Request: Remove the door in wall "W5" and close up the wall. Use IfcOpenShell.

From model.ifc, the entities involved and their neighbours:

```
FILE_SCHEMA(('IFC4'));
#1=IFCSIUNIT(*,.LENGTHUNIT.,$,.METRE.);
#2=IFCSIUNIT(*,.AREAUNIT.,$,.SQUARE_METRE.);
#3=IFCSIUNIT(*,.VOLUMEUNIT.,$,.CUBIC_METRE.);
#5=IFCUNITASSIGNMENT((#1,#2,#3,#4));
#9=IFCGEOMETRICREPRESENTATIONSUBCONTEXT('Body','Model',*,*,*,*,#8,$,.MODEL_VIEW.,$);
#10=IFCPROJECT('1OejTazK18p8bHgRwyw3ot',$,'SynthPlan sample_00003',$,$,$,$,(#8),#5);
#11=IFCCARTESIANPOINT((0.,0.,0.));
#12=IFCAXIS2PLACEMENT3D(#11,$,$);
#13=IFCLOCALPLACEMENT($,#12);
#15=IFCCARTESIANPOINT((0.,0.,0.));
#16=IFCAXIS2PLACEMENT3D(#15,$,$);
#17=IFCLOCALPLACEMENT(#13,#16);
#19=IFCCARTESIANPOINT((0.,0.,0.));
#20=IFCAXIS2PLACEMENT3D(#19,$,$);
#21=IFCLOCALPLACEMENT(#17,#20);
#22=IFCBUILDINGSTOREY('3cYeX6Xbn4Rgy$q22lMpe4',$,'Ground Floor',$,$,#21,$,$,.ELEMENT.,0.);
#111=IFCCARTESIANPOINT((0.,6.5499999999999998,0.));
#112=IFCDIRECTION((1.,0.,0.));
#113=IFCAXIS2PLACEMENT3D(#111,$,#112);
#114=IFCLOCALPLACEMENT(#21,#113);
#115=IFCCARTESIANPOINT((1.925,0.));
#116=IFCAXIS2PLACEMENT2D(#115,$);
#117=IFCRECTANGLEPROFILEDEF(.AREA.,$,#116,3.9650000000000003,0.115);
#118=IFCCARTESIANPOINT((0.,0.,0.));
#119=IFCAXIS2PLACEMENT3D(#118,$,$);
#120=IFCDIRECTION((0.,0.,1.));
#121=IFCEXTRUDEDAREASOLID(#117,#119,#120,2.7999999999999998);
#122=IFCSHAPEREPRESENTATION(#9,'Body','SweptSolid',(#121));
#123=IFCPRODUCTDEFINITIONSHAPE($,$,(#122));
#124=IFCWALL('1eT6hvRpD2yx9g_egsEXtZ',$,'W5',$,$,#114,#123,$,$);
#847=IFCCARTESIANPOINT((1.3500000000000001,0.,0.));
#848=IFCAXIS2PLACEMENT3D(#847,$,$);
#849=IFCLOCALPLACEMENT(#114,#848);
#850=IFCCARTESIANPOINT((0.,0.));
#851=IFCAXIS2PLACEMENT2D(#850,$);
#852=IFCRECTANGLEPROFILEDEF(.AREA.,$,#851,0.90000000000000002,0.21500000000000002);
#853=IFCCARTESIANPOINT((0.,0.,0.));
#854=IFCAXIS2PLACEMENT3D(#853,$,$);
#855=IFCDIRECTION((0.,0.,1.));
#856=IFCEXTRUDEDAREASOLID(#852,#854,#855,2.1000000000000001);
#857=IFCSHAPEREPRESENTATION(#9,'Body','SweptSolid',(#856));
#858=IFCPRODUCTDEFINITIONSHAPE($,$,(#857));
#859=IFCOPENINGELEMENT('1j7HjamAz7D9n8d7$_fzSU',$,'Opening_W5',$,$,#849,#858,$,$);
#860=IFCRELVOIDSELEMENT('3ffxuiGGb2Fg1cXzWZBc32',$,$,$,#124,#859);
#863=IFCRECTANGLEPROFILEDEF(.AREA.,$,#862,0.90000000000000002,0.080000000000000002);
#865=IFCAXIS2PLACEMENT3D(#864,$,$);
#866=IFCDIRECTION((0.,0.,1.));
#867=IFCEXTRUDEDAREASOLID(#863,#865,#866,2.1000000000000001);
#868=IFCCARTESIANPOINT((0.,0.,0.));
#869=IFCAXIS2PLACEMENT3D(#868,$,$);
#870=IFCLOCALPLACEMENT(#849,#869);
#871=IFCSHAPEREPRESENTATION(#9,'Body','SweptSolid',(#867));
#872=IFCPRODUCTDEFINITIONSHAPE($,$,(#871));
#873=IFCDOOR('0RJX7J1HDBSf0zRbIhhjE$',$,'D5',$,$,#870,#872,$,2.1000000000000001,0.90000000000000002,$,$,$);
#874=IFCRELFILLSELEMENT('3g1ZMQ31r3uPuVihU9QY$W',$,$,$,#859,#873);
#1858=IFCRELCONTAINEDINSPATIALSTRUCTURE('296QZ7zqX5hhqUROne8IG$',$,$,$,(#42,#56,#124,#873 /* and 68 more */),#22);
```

```python
import ifcopenshell
import ifcopenshell.api.feature
import ifcopenshell.api.root
import ifcopenshell.geom
import ifcopenshell.util.shape

model = ifcopenshell.open("model.ifc")
settings = ifcopenshell.geom.settings()


def volume(element):
    """Net volume in cubic metres, openings subtracted."""
    shape = ifcopenshell.geom.create_shape(settings, element)
    return ifcopenshell.util.shape.get_volume(shape.geometry)


door = model.by_guid("0RJX7J1HDBSf0zRbIhhjE$")
opening = door.FillsVoids[0].RelatingOpeningElement
wall = opening.VoidsElements[0].RelatingBuildingElement
before = volume(wall)

ifcopenshell.api.root.remove_product(model, product=door)
ifcopenshell.api.feature.remove_feature(model, feature=opening)

after = volume(wall)

print(f"wall volume {before:.3f} -> {after:.3f} m3")

model.write("model_updated.ifc")
```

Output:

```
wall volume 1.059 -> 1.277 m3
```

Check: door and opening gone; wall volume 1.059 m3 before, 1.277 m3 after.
